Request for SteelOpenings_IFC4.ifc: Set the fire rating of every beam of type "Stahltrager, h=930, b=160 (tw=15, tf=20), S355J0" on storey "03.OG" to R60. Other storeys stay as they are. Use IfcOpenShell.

First a look at what the model holds.

```python
import ifcopenshell
import ifcopenshell.util.element

model = ifcopenshell.open("SteelOpenings_IFC4.ifc")
print(model.schema)
storey = next(s for s in model.by_type("IfcBuildingStorey") if s.Name == "03.OG")
beams = [e for e in ifcopenshell.util.element.get_decomposition(storey) if e.is_a("IfcBeam")]
seen = {}
for e in beams:
    element_type = ifcopenshell.util.element.get_type(e)
    key = (element_type.Name if element_type != e and element_type else None, ifcopenshell.util.element.get_pset(e, "Pset_BeamCommon", "FireRating"))
    seen[key] = seen.get(key, 0) + 1
for (name, value), count in sorted(seen.items(), key=str):
    print(count, "x", name, "|", value)
```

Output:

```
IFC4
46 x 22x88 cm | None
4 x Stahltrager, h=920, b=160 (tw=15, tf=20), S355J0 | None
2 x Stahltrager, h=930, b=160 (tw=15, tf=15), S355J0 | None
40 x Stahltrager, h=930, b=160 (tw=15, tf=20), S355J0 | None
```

```python
import ifcopenshell
import ifcopenshell.api.pset
import ifcopenshell.util.element

model = ifcopenshell.open("SteelOpenings_IFC4.ifc")

storey = next(s for s in model.by_type("IfcBuildingStorey") if s.Name == "03.OG")
beams = [e for e in ifcopenshell.util.element.get_decomposition(storey) if e.is_a("IfcBeam")]

count = 0
for e in beams:
    element_type = ifcopenshell.util.element.get_type(e)
    if element_type in (None, e) or element_type.Name != "Stahltrager, h=930, b=160 (tw=15, tf=20), S355J0":
        continue
    # add_pset returns the element's existing set when there is one.
    pset = ifcopenshell.api.pset.add_pset(model, product=e, name="Pset_BeamCommon")
    ifcopenshell.api.pset.edit_pset(model, pset=pset, properties={"FireRating": "R60"})
    count += 1

print(count, "beams updated")

model.write("SteelOpenings_IFC4_edited.ifc")
```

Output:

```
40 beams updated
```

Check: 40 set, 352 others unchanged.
